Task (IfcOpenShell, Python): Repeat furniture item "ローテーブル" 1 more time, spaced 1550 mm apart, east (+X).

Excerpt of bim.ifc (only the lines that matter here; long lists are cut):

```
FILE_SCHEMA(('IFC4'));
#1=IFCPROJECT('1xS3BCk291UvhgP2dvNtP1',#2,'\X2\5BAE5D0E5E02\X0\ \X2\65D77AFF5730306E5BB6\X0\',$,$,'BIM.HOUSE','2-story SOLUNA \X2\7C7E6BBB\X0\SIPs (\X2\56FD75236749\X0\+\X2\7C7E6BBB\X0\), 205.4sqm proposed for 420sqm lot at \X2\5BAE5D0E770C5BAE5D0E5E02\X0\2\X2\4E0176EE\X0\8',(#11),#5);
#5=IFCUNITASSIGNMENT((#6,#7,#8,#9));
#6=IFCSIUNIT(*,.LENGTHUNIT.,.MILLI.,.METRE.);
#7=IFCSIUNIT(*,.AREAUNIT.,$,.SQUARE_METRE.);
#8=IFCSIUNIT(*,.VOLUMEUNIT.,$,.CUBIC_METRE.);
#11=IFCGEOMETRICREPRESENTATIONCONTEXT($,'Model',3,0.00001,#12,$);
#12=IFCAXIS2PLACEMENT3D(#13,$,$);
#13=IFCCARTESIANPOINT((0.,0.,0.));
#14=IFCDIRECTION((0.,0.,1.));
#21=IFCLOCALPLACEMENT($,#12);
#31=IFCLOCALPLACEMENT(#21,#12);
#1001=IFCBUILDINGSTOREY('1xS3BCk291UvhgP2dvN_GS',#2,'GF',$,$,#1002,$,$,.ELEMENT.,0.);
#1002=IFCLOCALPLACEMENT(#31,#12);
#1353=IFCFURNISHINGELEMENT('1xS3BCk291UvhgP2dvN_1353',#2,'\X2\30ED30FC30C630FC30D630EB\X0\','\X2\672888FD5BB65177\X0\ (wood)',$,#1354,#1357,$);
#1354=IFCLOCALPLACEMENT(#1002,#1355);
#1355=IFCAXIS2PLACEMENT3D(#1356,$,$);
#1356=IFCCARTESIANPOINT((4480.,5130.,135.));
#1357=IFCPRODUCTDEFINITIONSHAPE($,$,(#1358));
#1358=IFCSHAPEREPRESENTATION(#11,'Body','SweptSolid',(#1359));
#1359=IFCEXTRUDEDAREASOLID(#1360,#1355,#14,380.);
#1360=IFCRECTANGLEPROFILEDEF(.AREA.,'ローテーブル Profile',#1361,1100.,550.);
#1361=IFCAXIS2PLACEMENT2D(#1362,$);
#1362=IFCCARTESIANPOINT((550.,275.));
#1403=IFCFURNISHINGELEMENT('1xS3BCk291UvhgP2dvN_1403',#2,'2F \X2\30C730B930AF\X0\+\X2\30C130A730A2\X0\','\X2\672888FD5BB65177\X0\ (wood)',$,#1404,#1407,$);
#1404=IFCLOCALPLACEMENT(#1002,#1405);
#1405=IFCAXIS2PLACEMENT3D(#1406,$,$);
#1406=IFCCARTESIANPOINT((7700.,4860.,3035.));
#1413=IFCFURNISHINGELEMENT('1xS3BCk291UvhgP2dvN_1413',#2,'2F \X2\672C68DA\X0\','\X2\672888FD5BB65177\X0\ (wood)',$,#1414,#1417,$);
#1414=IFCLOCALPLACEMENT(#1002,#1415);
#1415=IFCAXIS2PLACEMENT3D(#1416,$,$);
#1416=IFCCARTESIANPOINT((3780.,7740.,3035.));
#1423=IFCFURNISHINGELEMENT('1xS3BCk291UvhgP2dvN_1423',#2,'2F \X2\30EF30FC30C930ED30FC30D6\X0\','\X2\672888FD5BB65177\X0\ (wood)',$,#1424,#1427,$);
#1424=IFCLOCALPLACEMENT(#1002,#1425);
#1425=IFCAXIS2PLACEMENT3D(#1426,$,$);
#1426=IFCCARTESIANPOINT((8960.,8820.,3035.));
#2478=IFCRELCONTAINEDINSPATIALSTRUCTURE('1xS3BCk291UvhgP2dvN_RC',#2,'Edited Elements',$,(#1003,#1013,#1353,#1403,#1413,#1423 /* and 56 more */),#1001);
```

```python
import numpy as np
import ifcopenshell
import ifcopenshell.api.geometry
import ifcopenshell.api.root
import ifcopenshell.util.element
import ifcopenshell.util.placement

model = ifcopenshell.open("bim.ifc")


def reuse_history(source, copy):
    """copy_class also copies each property set's owner history, people and application; keep the originals."""
    for rel in copy.IsDefinedBy:
        if rel.is_a("IfcRelDefinesByProperties") and (history := rel.RelatingPropertyDefinition.OwnerHistory):
            rel.RelatingPropertyDefinition.OwnerHistory = source.OwnerHistory
            ifcopenshell.util.element.remove_deep2(model, history)


source = model.by_guid("1xS3BCk291UvhgP2dvN_1353")
base = ifcopenshell.util.placement.get_local_placement(source.ObjectPlacement)
step = np.array([1.0, 0.0, 0.0]) * 1550.0

for i in range(1, 2):
    copy = ifcopenshell.api.root.copy_class(model, product=source)
    copy.Representation = ifcopenshell.util.element.copy_deep(
        model, source.Representation, exclude=["IfcGeometricRepresentationContext", "IfcRepresentationMap"]
    )
    reuse_history(source, copy)
    matrix = base.copy()
    matrix[:3, 3] += i * step
    print("added at", matrix[:3, 3].round(3) + 0.0)
    ifcopenshell.api.geometry.edit_object_placement(model, product=copy, matrix=matrix, is_si=False)

model.write("bim_edited.ifc")
```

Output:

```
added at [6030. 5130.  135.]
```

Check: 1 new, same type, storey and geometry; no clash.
